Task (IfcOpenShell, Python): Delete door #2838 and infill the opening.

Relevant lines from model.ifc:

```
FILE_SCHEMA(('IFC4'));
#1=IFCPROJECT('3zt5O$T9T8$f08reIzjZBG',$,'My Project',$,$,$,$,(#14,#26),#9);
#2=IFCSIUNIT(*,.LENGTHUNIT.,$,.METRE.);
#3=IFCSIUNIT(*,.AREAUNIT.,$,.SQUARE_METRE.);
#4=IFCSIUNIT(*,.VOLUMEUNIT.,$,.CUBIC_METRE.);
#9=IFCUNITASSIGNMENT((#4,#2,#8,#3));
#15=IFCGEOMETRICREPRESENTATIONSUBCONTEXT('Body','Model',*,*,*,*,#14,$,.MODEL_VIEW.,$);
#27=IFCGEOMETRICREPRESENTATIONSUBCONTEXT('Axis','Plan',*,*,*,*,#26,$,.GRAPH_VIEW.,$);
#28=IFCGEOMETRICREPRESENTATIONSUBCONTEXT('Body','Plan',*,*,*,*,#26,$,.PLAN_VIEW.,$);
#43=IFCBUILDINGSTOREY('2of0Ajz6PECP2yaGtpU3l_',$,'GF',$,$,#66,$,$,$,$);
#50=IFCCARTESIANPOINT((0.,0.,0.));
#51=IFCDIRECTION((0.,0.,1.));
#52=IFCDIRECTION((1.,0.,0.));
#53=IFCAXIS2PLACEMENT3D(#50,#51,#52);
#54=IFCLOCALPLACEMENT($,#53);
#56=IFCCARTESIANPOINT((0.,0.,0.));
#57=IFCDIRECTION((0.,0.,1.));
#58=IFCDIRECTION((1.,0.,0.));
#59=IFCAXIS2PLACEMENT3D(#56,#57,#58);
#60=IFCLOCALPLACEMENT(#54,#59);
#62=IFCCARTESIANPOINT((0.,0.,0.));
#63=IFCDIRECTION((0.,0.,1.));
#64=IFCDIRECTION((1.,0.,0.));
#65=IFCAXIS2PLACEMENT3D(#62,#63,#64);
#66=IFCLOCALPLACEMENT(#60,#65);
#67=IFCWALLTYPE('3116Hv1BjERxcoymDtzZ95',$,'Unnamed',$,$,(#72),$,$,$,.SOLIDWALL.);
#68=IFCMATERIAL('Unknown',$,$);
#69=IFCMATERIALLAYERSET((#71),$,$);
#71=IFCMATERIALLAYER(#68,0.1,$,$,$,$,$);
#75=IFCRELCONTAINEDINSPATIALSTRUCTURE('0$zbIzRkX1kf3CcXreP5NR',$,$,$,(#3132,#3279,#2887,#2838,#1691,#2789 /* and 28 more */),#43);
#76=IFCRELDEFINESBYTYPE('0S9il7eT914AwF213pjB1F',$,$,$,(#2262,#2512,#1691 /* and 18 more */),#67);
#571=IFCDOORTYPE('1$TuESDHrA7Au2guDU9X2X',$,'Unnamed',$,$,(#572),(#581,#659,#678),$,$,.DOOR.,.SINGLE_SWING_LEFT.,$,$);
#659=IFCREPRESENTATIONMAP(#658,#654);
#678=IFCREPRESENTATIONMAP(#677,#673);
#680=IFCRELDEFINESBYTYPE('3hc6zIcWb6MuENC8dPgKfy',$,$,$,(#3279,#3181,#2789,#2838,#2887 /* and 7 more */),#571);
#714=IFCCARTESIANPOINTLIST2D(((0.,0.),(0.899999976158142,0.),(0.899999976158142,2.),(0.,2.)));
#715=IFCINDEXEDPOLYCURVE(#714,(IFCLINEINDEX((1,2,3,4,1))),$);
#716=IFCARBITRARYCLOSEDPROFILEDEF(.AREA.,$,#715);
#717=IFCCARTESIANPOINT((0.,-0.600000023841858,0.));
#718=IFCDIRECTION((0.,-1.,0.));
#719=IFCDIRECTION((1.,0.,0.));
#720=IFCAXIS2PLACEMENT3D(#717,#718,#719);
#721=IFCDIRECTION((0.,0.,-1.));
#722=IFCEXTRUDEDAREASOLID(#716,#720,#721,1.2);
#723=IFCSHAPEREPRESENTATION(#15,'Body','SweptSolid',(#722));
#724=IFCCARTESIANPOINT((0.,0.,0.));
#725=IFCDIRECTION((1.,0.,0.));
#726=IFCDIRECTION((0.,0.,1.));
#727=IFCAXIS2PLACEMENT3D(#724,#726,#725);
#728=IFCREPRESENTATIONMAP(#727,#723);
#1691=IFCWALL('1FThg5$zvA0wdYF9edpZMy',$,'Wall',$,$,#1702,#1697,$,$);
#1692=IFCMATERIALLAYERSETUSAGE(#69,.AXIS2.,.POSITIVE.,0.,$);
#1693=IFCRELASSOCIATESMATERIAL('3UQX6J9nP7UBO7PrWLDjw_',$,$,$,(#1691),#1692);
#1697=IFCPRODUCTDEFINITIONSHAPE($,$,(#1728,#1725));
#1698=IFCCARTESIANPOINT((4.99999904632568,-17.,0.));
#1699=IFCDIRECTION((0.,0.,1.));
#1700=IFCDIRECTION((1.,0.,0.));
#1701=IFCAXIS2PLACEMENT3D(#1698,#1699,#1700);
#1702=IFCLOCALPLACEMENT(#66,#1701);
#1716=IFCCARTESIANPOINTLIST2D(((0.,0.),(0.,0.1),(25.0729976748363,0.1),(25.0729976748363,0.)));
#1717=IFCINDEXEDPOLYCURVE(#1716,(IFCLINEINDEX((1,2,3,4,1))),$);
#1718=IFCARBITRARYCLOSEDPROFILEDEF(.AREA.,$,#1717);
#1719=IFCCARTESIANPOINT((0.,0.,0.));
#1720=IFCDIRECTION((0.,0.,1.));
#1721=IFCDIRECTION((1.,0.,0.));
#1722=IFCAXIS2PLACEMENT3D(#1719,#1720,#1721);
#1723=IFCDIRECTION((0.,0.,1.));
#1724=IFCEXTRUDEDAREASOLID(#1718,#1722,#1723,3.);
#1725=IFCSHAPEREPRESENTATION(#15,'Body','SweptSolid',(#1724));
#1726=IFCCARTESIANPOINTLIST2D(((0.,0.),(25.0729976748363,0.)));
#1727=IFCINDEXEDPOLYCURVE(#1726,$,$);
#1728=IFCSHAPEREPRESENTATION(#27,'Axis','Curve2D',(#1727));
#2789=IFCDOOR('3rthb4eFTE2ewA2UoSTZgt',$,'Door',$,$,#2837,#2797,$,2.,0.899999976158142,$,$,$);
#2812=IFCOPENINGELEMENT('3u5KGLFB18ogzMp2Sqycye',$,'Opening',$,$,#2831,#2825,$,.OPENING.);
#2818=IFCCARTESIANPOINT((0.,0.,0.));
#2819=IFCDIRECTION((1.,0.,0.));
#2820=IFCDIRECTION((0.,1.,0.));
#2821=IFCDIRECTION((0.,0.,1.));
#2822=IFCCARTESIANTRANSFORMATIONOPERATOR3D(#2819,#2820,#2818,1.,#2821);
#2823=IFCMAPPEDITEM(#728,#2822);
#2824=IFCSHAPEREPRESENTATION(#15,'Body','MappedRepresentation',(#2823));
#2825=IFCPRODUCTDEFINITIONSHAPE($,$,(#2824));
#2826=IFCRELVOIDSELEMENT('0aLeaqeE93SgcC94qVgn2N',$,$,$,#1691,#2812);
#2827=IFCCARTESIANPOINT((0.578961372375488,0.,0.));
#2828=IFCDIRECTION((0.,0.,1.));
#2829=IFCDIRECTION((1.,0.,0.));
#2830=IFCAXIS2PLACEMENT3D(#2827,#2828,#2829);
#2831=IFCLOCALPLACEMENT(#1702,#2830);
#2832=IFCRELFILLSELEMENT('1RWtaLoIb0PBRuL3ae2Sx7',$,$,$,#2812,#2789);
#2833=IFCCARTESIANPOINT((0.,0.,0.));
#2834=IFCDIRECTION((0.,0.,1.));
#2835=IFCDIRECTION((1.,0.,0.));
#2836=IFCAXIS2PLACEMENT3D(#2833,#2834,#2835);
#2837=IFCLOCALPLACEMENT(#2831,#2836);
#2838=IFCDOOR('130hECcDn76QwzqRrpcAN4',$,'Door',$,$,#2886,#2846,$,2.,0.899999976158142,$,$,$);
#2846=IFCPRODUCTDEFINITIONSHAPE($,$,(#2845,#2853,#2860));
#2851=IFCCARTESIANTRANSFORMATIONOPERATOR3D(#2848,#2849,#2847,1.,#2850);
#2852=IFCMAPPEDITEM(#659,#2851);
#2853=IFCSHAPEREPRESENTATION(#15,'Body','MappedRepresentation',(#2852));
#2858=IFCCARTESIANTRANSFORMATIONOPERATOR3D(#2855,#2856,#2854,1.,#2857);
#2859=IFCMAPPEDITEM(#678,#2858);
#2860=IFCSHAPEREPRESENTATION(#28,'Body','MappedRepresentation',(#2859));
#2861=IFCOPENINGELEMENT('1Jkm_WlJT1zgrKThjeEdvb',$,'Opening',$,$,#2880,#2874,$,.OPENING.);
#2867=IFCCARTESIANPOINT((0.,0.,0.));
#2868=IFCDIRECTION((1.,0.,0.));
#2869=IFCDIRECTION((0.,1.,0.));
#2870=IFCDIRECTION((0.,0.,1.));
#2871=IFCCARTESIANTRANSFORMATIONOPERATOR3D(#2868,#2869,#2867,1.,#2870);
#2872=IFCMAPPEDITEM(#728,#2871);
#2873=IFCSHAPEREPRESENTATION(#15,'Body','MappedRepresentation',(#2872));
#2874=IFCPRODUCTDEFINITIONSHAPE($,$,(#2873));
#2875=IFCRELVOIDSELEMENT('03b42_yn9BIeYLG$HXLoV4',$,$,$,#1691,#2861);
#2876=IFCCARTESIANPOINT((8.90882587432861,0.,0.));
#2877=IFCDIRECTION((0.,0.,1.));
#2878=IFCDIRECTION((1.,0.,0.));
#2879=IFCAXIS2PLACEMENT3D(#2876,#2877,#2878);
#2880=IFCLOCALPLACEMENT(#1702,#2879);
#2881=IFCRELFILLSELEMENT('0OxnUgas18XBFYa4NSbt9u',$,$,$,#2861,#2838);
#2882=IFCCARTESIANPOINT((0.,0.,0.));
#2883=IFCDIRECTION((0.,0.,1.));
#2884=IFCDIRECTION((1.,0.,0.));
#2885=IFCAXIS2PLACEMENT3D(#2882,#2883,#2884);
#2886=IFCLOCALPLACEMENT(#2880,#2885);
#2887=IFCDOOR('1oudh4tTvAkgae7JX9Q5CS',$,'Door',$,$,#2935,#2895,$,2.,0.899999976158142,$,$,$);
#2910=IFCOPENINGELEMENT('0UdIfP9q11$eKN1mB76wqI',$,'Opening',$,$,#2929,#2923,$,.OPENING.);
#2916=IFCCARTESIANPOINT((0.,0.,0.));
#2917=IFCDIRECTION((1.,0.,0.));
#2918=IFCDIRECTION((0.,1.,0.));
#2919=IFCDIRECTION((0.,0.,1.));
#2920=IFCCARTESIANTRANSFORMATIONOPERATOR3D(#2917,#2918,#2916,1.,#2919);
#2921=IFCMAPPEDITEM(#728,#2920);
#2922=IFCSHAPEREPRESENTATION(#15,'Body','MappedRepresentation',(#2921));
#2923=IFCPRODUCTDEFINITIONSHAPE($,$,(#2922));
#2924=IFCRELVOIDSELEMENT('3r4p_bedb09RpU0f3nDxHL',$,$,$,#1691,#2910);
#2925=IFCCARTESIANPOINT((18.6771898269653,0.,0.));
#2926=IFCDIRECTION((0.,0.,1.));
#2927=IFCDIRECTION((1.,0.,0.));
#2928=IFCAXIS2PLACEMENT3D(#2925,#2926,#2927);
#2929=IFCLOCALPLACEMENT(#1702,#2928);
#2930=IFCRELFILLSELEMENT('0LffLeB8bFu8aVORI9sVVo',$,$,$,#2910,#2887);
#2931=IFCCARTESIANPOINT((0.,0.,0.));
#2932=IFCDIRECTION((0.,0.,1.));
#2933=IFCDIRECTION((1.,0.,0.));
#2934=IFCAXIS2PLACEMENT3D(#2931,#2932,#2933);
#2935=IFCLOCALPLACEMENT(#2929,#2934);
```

```python
import ifcopenshell
import ifcopenshell.api.feature
import ifcopenshell.api.root
import ifcopenshell.geom
import ifcopenshell.util.shape

model = ifcopenshell.open("model.ifc")
settings = ifcopenshell.geom.settings()


def volume(element):
    """Net volume in cubic metres, openings subtracted."""
    shape = ifcopenshell.geom.create_shape(settings, element)
    return ifcopenshell.util.shape.get_volume(shape.geometry)


door = model.by_guid("130hECcDn76QwzqRrpcAN4")
opening = door.FillsVoids[0].RelatingOpeningElement
wall = opening.VoidsElements[0].RelatingBuildingElement
before = volume(wall)

ifcopenshell.api.root.remove_product(model, product=door)
ifcopenshell.api.feature.remove_feature(model, feature=opening)

after = volume(wall)

print(f"wall volume {before:.3f} -> {after:.3f} m3")

model.write("model-out.ifc")
```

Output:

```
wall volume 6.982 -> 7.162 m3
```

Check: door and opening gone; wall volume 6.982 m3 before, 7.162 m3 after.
